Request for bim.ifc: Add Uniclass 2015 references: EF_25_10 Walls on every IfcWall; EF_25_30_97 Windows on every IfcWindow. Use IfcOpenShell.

First a look at what the model holds.

```python
import ifcopenshell

model = ifcopenshell.open("bim.ifc")
print(model.schema)
print("classifications:", [c.Name for c in model.by_type("IfcClassification")])
for ifc_class in ("IfcDoor", "IfcRoof", "IfcStair", "IfcWall", "IfcWindow"):
    print(ifc_class, len(model.by_type(ifc_class)))
```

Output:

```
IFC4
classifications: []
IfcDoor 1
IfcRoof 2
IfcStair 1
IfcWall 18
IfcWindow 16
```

```python
import ifcopenshell
import ifcopenshell.api.classification

model = ifcopenshell.open("bim.ifc")

system = ifcopenshell.api.classification.add_classification(model, classification="Uniclass 2015")

codes = {
    "IfcWall": ("EF_25_10", "Walls"),
    "IfcWindow": ("EF_25_30_97", "Windows"),
}
for ifc_class, (code, name) in codes.items():
    products = model.by_type(ifc_class)
    ifcopenshell.api.classification.add_reference(
        model, products=products, classification=system, identification=code, name=name
    )
    print(code, len(products))

model.write("bim_updated.ifc")
```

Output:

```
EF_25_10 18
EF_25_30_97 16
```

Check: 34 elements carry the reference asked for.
